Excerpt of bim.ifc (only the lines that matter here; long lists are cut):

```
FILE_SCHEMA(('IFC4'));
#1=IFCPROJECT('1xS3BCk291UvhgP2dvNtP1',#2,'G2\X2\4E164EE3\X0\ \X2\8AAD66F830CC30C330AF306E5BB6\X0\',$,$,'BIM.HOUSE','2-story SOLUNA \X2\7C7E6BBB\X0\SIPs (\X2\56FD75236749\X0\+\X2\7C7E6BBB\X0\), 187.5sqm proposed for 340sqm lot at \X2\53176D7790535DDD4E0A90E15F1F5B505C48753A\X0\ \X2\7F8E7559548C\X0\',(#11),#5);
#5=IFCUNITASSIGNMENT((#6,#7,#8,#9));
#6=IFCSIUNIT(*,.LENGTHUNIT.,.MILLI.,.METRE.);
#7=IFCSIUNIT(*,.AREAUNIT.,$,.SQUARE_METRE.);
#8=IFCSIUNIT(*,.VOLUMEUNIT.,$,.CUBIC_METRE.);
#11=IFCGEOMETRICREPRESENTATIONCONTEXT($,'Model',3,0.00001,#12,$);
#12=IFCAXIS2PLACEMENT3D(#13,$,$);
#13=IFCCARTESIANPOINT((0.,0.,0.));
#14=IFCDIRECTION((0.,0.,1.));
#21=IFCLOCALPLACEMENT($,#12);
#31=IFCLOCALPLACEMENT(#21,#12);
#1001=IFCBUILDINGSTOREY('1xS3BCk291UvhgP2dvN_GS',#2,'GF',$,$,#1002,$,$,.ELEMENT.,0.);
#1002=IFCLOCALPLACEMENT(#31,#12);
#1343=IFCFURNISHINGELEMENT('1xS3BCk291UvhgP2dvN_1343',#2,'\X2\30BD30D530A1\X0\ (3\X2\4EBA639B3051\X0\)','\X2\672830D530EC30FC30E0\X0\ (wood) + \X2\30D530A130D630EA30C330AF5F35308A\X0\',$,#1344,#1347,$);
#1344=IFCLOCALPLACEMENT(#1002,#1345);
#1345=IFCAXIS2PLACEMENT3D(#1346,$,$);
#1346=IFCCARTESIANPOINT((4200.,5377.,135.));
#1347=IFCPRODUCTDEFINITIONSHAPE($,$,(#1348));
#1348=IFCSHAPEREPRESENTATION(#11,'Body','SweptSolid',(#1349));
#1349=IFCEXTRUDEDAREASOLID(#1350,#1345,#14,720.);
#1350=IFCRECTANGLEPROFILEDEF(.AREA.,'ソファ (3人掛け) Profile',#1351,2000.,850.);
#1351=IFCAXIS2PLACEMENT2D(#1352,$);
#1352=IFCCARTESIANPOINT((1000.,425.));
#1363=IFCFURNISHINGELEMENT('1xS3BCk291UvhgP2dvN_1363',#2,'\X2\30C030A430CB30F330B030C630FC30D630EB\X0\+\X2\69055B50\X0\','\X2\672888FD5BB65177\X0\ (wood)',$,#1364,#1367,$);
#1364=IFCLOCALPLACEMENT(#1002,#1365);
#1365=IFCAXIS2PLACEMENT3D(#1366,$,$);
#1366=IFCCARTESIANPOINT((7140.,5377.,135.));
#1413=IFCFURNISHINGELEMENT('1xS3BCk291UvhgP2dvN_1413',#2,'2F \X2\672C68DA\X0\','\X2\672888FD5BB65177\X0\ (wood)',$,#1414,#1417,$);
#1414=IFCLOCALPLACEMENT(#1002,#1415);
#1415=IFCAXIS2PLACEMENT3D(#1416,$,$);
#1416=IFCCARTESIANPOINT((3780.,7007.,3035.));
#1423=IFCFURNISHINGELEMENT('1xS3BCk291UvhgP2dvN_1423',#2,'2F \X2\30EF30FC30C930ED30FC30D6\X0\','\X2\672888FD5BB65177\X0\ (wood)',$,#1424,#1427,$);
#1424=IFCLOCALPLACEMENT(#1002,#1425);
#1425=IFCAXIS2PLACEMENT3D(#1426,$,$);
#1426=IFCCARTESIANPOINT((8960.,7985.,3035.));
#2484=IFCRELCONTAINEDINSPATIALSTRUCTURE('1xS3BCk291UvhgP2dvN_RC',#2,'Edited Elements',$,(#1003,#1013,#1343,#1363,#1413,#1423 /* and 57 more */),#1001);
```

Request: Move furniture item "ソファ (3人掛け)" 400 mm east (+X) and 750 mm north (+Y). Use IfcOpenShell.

```python
import ifcopenshell
import ifcopenshell.api.geometry
import ifcopenshell.util.placement
import ifcopenshell.util.unit

model = ifcopenshell.open("bim.ifc")
unit_scale = ifcopenshell.util.unit.calculate_unit_scale(model)

item = model.by_guid("1xS3BCk291UvhgP2dvN_1343")
matrix = ifcopenshell.util.placement.get_local_placement(item.ObjectPlacement)
matrix[0, 3] += 0.4 / unit_scale
matrix[1, 3] += 0.75 / unit_scale
ifcopenshell.api.geometry.edit_object_placement(model, product=item, matrix=matrix, is_si=False)

print(ifcopenshell.util.placement.get_local_placement(item.ObjectPlacement).round(3) + 0.0)

model.write("bim_v2.ifc")
```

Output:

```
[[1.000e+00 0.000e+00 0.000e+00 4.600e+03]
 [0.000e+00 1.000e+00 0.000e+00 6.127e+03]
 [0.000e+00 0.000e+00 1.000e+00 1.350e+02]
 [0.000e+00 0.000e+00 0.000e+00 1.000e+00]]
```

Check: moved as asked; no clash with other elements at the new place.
